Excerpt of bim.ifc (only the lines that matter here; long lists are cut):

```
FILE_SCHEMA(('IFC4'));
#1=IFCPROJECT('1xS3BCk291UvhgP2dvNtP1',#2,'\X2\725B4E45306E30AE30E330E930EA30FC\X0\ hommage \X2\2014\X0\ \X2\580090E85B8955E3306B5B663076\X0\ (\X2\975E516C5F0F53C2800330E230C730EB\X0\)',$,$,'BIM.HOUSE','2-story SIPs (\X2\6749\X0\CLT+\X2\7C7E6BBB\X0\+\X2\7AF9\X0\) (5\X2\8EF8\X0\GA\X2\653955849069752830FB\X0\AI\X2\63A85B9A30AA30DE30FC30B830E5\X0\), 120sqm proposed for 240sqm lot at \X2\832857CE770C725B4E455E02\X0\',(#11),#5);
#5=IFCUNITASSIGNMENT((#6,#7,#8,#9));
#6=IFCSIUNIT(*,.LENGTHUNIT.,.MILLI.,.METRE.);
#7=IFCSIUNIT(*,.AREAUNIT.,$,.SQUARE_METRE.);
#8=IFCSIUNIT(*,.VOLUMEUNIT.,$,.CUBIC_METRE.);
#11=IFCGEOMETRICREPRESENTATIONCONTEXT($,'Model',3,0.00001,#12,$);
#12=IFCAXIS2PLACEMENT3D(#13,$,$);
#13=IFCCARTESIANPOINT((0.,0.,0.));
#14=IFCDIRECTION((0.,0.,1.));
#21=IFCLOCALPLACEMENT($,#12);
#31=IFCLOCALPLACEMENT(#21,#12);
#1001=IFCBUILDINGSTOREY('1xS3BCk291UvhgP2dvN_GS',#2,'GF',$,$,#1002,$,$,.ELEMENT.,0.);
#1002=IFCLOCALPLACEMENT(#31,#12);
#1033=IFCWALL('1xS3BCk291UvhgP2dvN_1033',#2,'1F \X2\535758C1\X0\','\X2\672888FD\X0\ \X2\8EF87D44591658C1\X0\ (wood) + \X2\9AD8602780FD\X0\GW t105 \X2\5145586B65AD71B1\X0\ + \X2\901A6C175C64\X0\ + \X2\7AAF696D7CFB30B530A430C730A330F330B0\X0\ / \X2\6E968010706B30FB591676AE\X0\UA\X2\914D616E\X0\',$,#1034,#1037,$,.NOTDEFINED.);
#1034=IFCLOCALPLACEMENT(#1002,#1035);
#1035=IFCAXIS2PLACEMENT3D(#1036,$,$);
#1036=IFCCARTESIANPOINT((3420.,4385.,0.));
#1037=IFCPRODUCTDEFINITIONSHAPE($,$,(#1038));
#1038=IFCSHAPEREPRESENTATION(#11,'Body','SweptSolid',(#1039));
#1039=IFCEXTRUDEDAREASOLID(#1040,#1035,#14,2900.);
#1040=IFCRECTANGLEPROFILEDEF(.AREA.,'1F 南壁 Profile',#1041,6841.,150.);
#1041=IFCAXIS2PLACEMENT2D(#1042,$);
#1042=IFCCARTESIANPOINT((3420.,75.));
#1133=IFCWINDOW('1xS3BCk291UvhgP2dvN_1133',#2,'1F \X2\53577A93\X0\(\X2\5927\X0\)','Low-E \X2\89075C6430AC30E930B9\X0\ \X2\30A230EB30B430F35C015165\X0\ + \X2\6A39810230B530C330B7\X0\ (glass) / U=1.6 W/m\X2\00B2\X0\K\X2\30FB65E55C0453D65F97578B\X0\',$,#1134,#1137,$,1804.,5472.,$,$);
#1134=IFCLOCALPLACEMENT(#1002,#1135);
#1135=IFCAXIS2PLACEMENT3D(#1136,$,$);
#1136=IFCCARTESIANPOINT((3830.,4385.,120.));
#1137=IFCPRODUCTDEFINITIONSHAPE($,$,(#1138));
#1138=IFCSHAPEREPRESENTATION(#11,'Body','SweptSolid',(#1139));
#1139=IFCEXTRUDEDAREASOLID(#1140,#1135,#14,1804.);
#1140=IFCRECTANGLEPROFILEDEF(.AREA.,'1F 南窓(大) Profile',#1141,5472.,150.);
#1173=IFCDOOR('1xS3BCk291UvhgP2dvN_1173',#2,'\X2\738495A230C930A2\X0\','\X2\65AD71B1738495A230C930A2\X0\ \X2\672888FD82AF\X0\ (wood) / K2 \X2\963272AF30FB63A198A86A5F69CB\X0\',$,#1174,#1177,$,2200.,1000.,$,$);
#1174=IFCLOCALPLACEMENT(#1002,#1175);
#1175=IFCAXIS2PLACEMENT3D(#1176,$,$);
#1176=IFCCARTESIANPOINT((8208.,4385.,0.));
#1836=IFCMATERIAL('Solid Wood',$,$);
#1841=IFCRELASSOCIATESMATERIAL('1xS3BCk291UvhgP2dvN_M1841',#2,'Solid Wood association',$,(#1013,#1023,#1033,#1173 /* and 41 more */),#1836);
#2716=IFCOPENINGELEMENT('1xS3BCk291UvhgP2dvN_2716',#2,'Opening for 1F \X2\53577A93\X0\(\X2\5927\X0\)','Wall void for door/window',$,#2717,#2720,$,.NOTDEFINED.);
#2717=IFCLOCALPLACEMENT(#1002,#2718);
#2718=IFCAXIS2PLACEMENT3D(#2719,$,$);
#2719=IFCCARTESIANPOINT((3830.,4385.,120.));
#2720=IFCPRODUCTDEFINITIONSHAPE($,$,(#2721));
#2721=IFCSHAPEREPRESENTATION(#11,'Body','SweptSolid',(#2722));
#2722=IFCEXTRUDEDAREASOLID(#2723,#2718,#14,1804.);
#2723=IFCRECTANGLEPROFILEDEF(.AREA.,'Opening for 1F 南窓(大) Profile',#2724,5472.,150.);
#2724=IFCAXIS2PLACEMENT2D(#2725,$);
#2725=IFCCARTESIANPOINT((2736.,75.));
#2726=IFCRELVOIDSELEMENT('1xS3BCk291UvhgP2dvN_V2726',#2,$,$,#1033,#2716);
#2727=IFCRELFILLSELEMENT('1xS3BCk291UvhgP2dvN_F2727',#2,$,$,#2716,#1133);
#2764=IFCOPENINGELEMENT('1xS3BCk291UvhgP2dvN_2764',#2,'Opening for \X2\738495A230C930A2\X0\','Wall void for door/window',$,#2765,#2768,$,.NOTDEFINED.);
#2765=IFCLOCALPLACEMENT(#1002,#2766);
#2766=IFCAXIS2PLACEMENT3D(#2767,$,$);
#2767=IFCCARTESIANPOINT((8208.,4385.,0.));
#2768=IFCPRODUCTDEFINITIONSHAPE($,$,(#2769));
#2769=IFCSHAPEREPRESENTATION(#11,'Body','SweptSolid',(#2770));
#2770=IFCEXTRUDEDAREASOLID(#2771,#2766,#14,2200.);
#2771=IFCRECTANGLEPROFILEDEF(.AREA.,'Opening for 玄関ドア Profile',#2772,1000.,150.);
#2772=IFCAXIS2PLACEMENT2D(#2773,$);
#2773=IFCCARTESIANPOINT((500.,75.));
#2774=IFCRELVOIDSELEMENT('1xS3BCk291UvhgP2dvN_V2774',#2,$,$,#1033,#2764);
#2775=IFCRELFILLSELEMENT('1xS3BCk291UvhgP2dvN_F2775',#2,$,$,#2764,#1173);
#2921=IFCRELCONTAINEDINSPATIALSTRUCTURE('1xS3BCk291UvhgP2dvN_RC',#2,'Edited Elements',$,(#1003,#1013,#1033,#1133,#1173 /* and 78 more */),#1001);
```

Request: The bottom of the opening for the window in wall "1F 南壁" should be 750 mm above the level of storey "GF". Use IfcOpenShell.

```python
import numpy as np
import ifcopenshell
import ifcopenshell.api.geometry
import ifcopenshell.geom
import ifcopenshell.util.element
import ifcopenshell.util.placement
import ifcopenshell.util.shape
import ifcopenshell.util.unit

model = ifcopenshell.open("bim.ifc")
unit_scale = ifcopenshell.util.unit.calculate_unit_scale(model)

window = model.by_guid("1xS3BCk291UvhgP2dvN_1133")
opening = window.FillsVoids[0].RelatingOpeningElement
storey = ifcopenshell.util.element.get_container(window, ifc_class="IfcBuildingStorey")
level = ifcopenshell.util.placement.get_local_placement(storey.ObjectPlacement)[2, 3]

# The opening's origin need not be at the sill, so measure its lowest point.
shape = ifcopenshell.geom.create_shape(ifcopenshell.geom.settings(), opening)
bottom = ifcopenshell.util.shape.get_shape_bottom_elevation(shape, shape.geometry) / unit_scale
dz = level + 0.75 / unit_scale - bottom

shift = np.array([0.0, 0.0, dz])
# The window is not placed relative to its opening, so move both.
for product in (opening, window):
    matrix = ifcopenshell.util.placement.get_local_placement(product.ObjectPlacement)
    matrix[:3, 3] += shift
    ifcopenshell.api.geometry.edit_object_placement(model, product=product, matrix=matrix, is_si=False)

print(f"moved by {dz * unit_scale:+.3f} m")

model.write("bim-out.ifc")
```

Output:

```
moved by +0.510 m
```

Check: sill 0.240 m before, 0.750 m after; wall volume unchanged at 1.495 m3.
